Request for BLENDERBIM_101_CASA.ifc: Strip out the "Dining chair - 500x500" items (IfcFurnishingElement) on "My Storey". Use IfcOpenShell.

First a look at what the model holds.

```python
import ifcopenshell
import ifcopenshell.util.element

model = ifcopenshell.open("BLENDERBIM_101_CASA.ifc")
print(model.schema)
storey = next(s for s in model.by_type("IfcBuildingStorey") if s.Name == "My Storey")
furniture = [e for e in ifcopenshell.util.element.get_decomposition(storey) if e.is_a("IfcFurnishingElement")]
seen = {}
for e in furniture:
    element_type = ifcopenshell.util.element.get_type(e)
    name = element_type.Name if element_type not in (None, e) else None
    seen[name] = seen.get(name, 0) + 1
for name, count in sorted(seen.items(), key=str):
    print(count, "x", name)
```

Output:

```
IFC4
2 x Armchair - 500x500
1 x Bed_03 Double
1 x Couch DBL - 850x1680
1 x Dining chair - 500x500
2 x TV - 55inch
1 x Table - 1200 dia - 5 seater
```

```python
import ifcopenshell
import ifcopenshell.api.root
import ifcopenshell.util.element

model = ifcopenshell.open("BLENDERBIM_101_CASA.ifc")

storey = next(s for s in model.by_type("IfcBuildingStorey") if s.Name == "My Storey")
furniture = [e for e in ifcopenshell.util.element.get_decomposition(storey) if e.is_a("IfcFurnishingElement")]
targets = [e for e in furniture if (t := ifcopenshell.util.element.get_type(e)) not in (None, e) and t.Name == "Dining chair - 500x500"]

for e in targets:
    ifcopenshell.api.root.remove_product(model, product=e)
print(len(targets), "removed")

model.write("BLENDERBIM_101_CASA_edited.ifc")
```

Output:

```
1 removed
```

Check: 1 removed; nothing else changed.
